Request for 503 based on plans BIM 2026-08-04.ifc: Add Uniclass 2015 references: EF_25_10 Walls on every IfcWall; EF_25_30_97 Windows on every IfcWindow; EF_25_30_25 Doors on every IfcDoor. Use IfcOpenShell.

First a look at what the model holds.

```python
import ifcopenshell

model = ifcopenshell.open("503 based on plans BIM 2026-08-04.ifc")
print(model.schema)
print("classifications:", [c.Name for c in model.by_type("IfcClassification")])
for ifc_class in ("IfcDoor", "IfcRoof", "IfcStair", "IfcWall", "IfcWindow"):
    print(ifc_class, len(model.by_type(ifc_class)))
```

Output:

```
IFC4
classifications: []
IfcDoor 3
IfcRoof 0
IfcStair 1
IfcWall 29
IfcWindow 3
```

```python
import ifcopenshell
import ifcopenshell.api.classification

model = ifcopenshell.open("503 based on plans BIM 2026-08-04.ifc")

system = ifcopenshell.api.classification.add_classification(model, classification="Uniclass 2015")

codes = {
    "IfcWall": ("EF_25_10", "Walls"),
    "IfcWindow": ("EF_25_30_97", "Windows"),
    "IfcDoor": ("EF_25_30_25", "Doors"),
}
for ifc_class, (code, name) in codes.items():
    products = model.by_type(ifc_class)
    ifcopenshell.api.classification.add_reference(
        model, products=products, classification=system, identification=code, name=name
    )
    print(code, len(products))

model.write("503 based on plans BIM 2026-08-04_edited.ifc")
```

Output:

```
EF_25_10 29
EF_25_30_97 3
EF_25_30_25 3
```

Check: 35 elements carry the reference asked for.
